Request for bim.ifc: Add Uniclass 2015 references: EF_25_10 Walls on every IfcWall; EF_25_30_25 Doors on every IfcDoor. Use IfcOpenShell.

First a look at what the model holds.

```python
import ifcopenshell

model = ifcopenshell.open("bim.ifc")
print(model.schema)
print("classifications:", [c.Name for c in model.by_type("IfcClassification")])
for ifc_class in ("IfcDoor", "IfcRoof", "IfcStair", "IfcWall", "IfcWindow"):
    print(ifc_class, len(model.by_type(ifc_class)))
```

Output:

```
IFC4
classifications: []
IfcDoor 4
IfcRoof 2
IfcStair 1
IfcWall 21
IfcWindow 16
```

```python
import ifcopenshell
import ifcopenshell.api.classification

model = ifcopenshell.open("bim.ifc")

system = ifcopenshell.api.classification.add_classification(model, classification="Uniclass 2015")

codes = {
    "IfcWall": ("EF_25_10", "Walls"),
    "IfcDoor": ("EF_25_30_25", "Doors"),
}
for ifc_class, (code, name) in codes.items():
    products = model.by_type(ifc_class)
    ifcopenshell.api.classification.add_reference(
        model, products=products, classification=system, identification=code, name=name
    )
    print(code, len(products))

model.write("bim_v2.ifc")
```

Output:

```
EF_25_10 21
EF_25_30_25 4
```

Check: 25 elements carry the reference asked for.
